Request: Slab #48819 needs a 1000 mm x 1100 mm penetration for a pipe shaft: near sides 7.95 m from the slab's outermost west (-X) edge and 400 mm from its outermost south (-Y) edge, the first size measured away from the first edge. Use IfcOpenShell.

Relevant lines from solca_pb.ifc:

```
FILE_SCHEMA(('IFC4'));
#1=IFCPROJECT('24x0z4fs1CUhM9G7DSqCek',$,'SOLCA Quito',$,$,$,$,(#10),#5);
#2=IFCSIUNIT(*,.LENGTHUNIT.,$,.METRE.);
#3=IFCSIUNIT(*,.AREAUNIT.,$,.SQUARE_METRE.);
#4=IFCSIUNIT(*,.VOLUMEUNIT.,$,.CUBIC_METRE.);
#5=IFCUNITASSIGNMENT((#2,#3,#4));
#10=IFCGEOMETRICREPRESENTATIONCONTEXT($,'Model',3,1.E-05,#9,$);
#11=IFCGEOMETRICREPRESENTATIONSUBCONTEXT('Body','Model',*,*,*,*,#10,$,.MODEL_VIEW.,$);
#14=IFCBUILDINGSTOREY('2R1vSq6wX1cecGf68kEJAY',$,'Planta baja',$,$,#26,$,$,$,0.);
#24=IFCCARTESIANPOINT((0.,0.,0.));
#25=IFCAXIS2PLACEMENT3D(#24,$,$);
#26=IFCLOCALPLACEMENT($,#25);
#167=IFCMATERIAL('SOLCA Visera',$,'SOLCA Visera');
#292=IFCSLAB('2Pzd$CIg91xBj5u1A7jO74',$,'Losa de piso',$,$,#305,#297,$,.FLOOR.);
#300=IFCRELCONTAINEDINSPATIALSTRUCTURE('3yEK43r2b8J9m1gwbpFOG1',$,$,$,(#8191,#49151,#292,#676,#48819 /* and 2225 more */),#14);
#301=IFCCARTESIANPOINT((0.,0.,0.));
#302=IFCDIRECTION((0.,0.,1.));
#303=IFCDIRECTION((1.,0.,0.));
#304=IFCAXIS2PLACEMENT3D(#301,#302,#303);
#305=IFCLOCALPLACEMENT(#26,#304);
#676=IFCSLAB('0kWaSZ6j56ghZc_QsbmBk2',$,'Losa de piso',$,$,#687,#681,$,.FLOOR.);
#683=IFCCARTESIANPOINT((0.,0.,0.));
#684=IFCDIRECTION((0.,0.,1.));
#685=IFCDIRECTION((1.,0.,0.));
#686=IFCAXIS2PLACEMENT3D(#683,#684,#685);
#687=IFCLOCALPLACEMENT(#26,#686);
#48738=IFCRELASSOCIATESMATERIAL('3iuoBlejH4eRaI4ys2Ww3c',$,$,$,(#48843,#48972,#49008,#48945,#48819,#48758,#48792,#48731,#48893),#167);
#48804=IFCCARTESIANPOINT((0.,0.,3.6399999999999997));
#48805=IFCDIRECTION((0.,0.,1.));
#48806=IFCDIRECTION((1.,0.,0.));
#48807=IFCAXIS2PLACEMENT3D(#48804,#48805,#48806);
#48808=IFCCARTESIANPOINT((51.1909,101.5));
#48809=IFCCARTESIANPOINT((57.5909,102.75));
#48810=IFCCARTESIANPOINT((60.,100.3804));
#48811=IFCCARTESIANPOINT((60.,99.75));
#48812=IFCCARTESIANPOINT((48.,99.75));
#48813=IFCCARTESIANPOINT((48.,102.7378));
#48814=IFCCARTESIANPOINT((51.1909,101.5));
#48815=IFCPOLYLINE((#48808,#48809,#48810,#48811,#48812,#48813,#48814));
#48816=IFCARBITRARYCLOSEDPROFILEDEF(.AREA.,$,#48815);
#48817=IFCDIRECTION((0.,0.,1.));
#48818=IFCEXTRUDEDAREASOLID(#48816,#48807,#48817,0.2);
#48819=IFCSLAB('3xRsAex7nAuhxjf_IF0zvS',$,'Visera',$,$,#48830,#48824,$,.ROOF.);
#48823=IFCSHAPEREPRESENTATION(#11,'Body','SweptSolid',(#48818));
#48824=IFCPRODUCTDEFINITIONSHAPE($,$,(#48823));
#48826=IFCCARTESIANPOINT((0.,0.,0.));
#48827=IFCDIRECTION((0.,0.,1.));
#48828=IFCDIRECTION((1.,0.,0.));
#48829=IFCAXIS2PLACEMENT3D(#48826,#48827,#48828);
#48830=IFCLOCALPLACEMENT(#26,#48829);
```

```python
import numpy as np
import ifcopenshell
import ifcopenshell.api.feature
import ifcopenshell.api.geometry
import ifcopenshell.api.root
import ifcopenshell.geom
import ifcopenshell.util.placement
import ifcopenshell.util.representation
import ifcopenshell.util.shape
import ifcopenshell.util.unit

model = ifcopenshell.open("solca_pb.ifc")
unit_scale = ifcopenshell.util.unit.calculate_unit_scale(model)
settings = ifcopenshell.geom.settings()


def volume(element):
    """Net volume in cubic metres, openings subtracted."""
    shape = ifcopenshell.geom.create_shape(settings, element)
    return ifcopenshell.util.shape.get_volume(shape.geometry)


slab = model.by_guid("3xRsAex7nAuhxjf_IF0zvS")
before = volume(slab)

# Extent in the slab's own axes, in metres. The edges named are its -X and -Y sides.
slab_shape = ifcopenshell.geom.create_shape(settings, slab)
vertices = ifcopenshell.util.shape.get_vertices(slab_shape.geometry)
x_min, y_min, bottom = vertices.min(axis=0)
top = vertices[:, 2].max()

opening = ifcopenshell.api.root.create_entity(model, ifc_class="IfcOpeningElement", name="Pipe shaft opening", predefined_type="OPENING")
context = ifcopenshell.util.representation.get_context(model, "Model", "Body", "MODEL_VIEW")
width, depth = 1, 1.1
outline = [(0.0, 0.0), (width, 0.0), (width, depth), (0.0, depth), (0.0, 0.0)]
# Overshoot both faces by 50 mm so the cut is clean.
shape = ifcopenshell.api.geometry.add_slab_representation(
    model, context=context, depth=top - bottom + 0.1, polyline=outline
)
ifcopenshell.api.geometry.assign_representation(model, product=opening, representation=shape)

matrix = ifcopenshell.util.placement.get_local_placement(slab.ObjectPlacement)
matrix[:, 3] = matrix @ np.append(np.array([x_min + 7.95, y_min + 0.4, bottom - 0.05]) / unit_scale, 1.0)
ifcopenshell.api.geometry.edit_object_placement(model, product=opening, matrix=matrix, is_si=False)
ifcopenshell.api.feature.add_feature(model, feature=opening, element=slab)

after = volume(slab)

print(f"slab volume {before:.3f} -> {after:.3f} m3")

model.write("solca_pb_updated.ifc")
```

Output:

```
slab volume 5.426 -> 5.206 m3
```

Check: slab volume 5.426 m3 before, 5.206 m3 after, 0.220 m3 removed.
